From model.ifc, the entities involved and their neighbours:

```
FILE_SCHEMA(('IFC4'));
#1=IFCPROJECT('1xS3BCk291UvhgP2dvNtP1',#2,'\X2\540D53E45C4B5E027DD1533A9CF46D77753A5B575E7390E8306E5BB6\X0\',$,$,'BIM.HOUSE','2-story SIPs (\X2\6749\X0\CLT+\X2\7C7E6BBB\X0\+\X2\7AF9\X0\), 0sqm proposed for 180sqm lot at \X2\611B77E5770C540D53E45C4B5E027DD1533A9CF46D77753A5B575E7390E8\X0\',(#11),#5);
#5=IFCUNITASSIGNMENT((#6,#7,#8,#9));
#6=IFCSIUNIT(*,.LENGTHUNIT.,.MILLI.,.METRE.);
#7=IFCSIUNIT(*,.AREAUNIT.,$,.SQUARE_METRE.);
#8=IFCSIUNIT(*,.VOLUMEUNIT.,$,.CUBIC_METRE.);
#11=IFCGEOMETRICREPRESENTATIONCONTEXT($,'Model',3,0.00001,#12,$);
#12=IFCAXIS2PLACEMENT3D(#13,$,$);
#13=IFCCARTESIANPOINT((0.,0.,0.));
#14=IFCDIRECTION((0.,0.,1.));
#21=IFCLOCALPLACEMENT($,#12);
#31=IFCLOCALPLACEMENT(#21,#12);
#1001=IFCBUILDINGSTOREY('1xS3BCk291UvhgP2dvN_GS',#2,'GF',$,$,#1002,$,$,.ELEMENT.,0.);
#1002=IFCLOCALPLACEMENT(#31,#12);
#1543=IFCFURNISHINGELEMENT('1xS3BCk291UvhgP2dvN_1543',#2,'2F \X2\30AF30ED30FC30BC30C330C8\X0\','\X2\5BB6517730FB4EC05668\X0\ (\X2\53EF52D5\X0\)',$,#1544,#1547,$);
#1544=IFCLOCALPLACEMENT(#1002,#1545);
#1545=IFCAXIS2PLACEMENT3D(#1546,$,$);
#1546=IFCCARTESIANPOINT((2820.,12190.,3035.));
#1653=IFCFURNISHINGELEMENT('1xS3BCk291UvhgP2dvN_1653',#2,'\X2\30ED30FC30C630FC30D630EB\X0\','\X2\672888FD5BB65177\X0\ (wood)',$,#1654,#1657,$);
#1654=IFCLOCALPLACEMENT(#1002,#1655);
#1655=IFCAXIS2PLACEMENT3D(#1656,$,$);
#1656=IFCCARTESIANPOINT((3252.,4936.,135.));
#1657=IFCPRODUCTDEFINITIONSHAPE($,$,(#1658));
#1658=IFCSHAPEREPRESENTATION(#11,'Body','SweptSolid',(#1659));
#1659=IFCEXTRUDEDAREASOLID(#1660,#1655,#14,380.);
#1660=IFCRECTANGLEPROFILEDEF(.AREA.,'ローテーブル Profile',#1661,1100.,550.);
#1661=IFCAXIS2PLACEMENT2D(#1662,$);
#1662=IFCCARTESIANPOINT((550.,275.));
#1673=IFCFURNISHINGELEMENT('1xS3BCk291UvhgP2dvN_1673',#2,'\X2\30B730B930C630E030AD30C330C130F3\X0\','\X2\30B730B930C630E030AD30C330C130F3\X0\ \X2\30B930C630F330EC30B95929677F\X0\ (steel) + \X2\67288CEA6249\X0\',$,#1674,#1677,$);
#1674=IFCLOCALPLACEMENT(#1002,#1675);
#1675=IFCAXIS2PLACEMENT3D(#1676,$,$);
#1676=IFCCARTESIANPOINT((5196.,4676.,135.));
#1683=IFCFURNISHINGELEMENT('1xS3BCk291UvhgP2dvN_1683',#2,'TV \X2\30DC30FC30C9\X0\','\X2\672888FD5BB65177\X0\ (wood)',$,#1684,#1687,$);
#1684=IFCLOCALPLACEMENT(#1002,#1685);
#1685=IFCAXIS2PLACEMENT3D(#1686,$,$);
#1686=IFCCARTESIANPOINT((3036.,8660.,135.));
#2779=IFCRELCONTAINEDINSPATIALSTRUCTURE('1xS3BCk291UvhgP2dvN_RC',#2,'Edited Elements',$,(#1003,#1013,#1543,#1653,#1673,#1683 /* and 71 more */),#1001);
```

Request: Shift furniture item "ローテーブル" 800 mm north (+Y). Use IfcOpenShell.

```python
import ifcopenshell
import ifcopenshell.api.geometry
import ifcopenshell.util.placement
import ifcopenshell.util.unit

model = ifcopenshell.open("model.ifc")
unit_scale = ifcopenshell.util.unit.calculate_unit_scale(model)

item = model.by_guid("1xS3BCk291UvhgP2dvN_1653")
matrix = ifcopenshell.util.placement.get_local_placement(item.ObjectPlacement)
matrix[1, 3] += 0.8 / unit_scale
ifcopenshell.api.geometry.edit_object_placement(model, product=item, matrix=matrix, is_si=False)

print(ifcopenshell.util.placement.get_local_placement(item.ObjectPlacement).round(3) + 0.0)

model.write("model-out.ifc")
```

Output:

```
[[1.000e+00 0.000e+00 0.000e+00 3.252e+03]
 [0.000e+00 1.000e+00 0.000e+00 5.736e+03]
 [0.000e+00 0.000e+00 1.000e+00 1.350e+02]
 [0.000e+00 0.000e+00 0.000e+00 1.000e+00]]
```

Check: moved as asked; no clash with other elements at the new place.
